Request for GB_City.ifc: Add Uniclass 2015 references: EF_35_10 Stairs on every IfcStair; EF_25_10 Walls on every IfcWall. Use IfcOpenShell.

First a look at what the model holds.

```python
import ifcopenshell

model = ifcopenshell.open("GB_City.ifc")
print(model.schema)
print("classifications:", [c.Name for c in model.by_type("IfcClassification")])
for ifc_class in ("IfcDoor", "IfcRoof", "IfcStair", "IfcWall", "IfcWindow"):
    print(ifc_class, len(model.by_type(ifc_class)))
```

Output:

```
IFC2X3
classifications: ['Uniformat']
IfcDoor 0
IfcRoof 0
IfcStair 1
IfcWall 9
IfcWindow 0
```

```python
import ifcopenshell
import ifcopenshell.api.classification

model = ifcopenshell.open("GB_City.ifc")

# IFC2X3 requires Source and Edition and has no link from the project to the system.
system = model.create_entity("IfcClassification", Source="NBS", Edition="2015", Name="Uniclass 2015")

codes = {
    "IfcStair": ("EF_35_10", "Stairs"),
    "IfcWall": ("EF_25_10", "Walls"),
}
for ifc_class, (code, name) in codes.items():
    products = model.by_type(ifc_class)
    ifcopenshell.api.classification.add_reference(
        model, products=products, classification=system, identification=code, name=name
    )
    print(code, len(products))

model.write("GB_City_v2.ifc")
```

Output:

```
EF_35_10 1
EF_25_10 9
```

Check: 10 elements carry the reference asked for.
